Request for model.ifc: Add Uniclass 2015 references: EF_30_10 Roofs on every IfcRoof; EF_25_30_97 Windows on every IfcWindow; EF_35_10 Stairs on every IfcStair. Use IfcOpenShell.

First a look at what the model holds.

```python
import ifcopenshell

model = ifcopenshell.open("model.ifc")
print(model.schema)
print("classifications:", [c.Name for c in model.by_type("IfcClassification")])
for ifc_class in ("IfcDoor", "IfcRoof", "IfcStair", "IfcWall", "IfcWindow"):
    print(ifc_class, len(model.by_type(ifc_class)))
```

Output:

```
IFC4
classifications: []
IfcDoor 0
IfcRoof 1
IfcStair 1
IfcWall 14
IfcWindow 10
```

```python
import ifcopenshell
import ifcopenshell.api.classification

model = ifcopenshell.open("model.ifc")

system = ifcopenshell.api.classification.add_classification(model, classification="Uniclass 2015")

codes = {
    "IfcRoof": ("EF_30_10", "Roofs"),
    "IfcWindow": ("EF_25_30_97", "Windows"),
    "IfcStair": ("EF_35_10", "Stairs"),
}
for ifc_class, (code, name) in codes.items():
    products = model.by_type(ifc_class)
    ifcopenshell.api.classification.add_reference(
        model, products=products, classification=system, identification=code, name=name
    )
    print(code, len(products))

model.write("model_edited.ifc")
```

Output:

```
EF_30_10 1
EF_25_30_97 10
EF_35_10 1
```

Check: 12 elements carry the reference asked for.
